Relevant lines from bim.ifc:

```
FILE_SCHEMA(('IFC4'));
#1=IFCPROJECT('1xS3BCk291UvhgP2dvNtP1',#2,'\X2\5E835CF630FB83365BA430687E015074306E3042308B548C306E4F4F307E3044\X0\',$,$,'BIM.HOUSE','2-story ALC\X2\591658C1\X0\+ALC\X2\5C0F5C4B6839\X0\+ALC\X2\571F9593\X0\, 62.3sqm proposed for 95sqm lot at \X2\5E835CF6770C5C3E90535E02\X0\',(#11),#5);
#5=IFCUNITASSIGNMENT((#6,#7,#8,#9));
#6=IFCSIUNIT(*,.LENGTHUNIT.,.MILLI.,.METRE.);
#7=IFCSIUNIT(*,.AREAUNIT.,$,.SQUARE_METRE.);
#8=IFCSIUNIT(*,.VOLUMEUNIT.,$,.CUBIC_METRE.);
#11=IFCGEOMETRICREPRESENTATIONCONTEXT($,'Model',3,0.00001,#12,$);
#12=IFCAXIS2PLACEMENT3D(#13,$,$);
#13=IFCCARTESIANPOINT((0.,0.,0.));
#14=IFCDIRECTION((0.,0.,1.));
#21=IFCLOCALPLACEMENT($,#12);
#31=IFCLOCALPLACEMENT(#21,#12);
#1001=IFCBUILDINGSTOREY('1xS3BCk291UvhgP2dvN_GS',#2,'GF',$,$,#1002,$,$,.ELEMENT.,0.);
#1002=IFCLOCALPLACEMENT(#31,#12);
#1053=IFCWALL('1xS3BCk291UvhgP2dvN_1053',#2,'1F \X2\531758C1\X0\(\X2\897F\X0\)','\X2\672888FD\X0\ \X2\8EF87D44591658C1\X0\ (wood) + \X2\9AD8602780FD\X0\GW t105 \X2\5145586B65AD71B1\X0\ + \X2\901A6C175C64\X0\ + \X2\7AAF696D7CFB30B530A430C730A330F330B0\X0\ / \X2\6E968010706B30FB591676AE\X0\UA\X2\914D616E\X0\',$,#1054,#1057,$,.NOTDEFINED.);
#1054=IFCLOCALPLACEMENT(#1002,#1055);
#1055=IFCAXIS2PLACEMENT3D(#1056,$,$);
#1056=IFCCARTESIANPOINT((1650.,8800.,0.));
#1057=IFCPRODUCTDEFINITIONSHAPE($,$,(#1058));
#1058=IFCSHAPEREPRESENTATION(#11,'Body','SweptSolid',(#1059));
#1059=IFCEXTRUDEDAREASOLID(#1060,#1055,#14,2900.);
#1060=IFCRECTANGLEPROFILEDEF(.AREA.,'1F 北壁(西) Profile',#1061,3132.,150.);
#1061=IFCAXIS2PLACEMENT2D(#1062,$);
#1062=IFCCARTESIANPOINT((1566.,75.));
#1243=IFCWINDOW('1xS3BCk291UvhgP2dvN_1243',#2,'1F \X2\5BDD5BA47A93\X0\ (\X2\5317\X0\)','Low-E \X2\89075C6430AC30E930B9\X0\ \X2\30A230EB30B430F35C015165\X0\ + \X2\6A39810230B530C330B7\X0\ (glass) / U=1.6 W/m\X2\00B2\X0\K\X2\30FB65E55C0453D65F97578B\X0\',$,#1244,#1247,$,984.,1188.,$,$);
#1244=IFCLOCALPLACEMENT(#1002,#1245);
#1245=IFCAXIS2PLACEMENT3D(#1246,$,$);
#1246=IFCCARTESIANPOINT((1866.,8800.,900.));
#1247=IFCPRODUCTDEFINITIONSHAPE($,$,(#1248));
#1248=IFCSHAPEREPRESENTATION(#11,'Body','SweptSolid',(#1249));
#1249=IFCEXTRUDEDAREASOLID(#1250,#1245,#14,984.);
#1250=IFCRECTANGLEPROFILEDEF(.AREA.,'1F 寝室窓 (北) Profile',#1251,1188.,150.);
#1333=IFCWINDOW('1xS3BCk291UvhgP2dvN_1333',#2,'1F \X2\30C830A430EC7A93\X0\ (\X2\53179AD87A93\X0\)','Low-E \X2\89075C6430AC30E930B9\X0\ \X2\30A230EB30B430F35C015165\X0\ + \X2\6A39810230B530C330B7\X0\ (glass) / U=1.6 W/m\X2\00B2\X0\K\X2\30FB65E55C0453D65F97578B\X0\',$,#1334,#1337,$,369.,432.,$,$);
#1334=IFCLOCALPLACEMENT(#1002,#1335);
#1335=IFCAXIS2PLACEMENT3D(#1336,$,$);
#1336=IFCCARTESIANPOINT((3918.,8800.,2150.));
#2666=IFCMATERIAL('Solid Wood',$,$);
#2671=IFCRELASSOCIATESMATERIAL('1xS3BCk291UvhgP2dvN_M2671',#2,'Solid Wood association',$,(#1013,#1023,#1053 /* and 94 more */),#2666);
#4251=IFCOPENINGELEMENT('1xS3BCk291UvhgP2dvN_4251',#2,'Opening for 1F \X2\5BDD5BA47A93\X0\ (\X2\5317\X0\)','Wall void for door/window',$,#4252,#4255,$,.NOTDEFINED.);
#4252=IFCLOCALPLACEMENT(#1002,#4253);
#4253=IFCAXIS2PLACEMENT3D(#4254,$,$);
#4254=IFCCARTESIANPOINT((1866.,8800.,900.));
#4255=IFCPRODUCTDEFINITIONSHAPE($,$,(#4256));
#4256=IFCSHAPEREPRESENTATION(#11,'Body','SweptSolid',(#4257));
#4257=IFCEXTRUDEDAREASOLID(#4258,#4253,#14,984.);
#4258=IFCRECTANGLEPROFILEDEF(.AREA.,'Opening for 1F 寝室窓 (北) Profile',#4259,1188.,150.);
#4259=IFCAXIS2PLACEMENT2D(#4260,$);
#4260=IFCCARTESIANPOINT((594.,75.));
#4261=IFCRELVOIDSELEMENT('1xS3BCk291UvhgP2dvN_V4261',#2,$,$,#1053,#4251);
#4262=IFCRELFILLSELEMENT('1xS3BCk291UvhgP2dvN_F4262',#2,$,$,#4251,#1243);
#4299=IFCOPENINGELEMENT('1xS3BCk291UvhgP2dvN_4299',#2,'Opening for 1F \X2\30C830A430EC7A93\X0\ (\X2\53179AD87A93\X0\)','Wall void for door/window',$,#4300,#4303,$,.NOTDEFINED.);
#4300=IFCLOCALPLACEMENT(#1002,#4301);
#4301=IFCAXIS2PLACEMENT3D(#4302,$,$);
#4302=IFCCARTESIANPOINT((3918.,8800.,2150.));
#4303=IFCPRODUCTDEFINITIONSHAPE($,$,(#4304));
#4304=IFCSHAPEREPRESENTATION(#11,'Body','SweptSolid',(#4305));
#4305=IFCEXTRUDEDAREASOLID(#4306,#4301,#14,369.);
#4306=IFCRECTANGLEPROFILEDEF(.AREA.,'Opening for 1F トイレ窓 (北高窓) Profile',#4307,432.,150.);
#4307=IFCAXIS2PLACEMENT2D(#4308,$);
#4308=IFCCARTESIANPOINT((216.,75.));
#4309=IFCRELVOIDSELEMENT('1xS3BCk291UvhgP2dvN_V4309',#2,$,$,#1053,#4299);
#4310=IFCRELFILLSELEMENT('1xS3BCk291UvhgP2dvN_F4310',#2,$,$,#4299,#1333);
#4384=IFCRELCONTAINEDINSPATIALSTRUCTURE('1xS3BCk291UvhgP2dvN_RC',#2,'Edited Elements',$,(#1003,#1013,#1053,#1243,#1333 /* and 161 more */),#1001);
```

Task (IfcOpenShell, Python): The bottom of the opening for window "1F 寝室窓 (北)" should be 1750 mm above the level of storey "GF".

```python
import numpy as np
import ifcopenshell
import ifcopenshell.api.geometry
import ifcopenshell.geom
import ifcopenshell.util.element
import ifcopenshell.util.placement
import ifcopenshell.util.shape
import ifcopenshell.util.unit

model = ifcopenshell.open("bim.ifc")
unit_scale = ifcopenshell.util.unit.calculate_unit_scale(model)

window = model.by_guid("1xS3BCk291UvhgP2dvN_1243")
opening = window.FillsVoids[0].RelatingOpeningElement
storey = ifcopenshell.util.element.get_container(window, ifc_class="IfcBuildingStorey")
level = ifcopenshell.util.placement.get_local_placement(storey.ObjectPlacement)[2, 3]

# The opening's origin need not be at the sill, so measure its lowest point.
shape = ifcopenshell.geom.create_shape(ifcopenshell.geom.settings(), opening)
bottom = ifcopenshell.util.shape.get_shape_bottom_elevation(shape, shape.geometry) / unit_scale
dz = level + 1.75 / unit_scale - bottom

shift = np.array([0.0, 0.0, dz])
# The window is not placed relative to its opening, so move both.
for product in (opening, window):
    matrix = ifcopenshell.util.placement.get_local_placement(product.ObjectPlacement)
    matrix[:3, 3] += shift
    ifcopenshell.api.geometry.edit_object_placement(model, product=product, matrix=matrix, is_si=False)

print(f"moved by {dz * unit_scale:+.3f} m")

model.write("bim_updated.ifc")
```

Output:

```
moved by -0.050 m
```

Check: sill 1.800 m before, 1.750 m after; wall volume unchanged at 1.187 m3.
